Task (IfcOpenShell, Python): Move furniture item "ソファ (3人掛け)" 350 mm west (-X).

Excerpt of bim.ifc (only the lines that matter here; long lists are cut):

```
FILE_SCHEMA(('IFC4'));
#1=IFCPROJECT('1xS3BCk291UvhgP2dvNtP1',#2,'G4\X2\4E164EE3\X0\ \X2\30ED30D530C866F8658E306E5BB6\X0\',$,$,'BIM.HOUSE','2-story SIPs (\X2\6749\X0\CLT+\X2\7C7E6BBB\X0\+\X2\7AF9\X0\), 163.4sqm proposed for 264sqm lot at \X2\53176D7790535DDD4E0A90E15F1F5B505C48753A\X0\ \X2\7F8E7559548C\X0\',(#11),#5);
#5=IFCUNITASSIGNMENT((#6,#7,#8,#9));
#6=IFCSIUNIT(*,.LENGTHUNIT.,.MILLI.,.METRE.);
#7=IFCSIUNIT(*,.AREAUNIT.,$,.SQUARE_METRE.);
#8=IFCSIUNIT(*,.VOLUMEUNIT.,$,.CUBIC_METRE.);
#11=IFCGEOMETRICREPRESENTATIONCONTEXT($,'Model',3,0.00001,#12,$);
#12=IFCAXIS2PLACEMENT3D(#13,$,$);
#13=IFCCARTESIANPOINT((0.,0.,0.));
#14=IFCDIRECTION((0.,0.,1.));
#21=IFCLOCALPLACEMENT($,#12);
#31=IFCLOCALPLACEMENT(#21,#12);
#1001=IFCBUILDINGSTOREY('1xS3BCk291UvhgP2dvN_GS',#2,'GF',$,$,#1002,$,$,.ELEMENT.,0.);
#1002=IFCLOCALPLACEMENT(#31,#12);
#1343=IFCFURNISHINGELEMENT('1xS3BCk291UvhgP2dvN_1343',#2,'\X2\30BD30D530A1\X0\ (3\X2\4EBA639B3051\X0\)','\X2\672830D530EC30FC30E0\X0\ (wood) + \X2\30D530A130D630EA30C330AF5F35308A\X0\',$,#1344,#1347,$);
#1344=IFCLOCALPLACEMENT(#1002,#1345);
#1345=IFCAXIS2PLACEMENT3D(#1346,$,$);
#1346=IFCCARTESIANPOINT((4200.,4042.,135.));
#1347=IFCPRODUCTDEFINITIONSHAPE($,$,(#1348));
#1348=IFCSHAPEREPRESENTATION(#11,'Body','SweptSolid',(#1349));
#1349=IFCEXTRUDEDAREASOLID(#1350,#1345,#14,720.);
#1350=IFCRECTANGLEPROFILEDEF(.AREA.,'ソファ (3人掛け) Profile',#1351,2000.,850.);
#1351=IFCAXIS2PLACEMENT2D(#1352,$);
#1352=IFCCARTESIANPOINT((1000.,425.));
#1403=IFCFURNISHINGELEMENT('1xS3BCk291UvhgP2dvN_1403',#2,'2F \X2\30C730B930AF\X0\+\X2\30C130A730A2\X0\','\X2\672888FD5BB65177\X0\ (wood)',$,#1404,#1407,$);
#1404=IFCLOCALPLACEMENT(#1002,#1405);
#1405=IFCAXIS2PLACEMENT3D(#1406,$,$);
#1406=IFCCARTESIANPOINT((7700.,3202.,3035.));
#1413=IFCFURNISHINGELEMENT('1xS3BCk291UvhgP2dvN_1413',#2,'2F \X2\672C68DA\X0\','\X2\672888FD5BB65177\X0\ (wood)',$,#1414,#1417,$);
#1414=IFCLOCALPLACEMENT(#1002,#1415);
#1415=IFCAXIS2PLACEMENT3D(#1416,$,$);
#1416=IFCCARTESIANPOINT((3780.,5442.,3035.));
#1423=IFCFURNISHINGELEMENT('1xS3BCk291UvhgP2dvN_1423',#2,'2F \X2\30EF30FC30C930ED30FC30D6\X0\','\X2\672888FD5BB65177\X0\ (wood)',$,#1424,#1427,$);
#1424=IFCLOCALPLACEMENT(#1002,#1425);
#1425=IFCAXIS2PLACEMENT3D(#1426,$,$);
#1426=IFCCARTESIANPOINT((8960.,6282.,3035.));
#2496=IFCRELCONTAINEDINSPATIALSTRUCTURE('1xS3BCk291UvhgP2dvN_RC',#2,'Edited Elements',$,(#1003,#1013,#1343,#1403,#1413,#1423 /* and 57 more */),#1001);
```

```python
import ifcopenshell
import ifcopenshell.api.geometry
import ifcopenshell.util.placement

model = ifcopenshell.open("bim.ifc")

item = model.by_guid("1xS3BCk291UvhgP2dvN_1343")
matrix = ifcopenshell.util.placement.get_local_placement(item.ObjectPlacement)
matrix[0, 3] -= 350.0
ifcopenshell.api.geometry.edit_object_placement(model, product=item, matrix=matrix, is_si=False)

print(ifcopenshell.util.placement.get_local_placement(item.ObjectPlacement).round(3) + 0.0)

model.write("bim_edited.ifc")
```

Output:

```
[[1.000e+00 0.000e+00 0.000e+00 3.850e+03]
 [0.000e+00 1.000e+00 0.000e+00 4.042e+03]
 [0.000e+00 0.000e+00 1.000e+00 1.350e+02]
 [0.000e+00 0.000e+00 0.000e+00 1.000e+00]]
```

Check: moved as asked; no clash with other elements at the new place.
